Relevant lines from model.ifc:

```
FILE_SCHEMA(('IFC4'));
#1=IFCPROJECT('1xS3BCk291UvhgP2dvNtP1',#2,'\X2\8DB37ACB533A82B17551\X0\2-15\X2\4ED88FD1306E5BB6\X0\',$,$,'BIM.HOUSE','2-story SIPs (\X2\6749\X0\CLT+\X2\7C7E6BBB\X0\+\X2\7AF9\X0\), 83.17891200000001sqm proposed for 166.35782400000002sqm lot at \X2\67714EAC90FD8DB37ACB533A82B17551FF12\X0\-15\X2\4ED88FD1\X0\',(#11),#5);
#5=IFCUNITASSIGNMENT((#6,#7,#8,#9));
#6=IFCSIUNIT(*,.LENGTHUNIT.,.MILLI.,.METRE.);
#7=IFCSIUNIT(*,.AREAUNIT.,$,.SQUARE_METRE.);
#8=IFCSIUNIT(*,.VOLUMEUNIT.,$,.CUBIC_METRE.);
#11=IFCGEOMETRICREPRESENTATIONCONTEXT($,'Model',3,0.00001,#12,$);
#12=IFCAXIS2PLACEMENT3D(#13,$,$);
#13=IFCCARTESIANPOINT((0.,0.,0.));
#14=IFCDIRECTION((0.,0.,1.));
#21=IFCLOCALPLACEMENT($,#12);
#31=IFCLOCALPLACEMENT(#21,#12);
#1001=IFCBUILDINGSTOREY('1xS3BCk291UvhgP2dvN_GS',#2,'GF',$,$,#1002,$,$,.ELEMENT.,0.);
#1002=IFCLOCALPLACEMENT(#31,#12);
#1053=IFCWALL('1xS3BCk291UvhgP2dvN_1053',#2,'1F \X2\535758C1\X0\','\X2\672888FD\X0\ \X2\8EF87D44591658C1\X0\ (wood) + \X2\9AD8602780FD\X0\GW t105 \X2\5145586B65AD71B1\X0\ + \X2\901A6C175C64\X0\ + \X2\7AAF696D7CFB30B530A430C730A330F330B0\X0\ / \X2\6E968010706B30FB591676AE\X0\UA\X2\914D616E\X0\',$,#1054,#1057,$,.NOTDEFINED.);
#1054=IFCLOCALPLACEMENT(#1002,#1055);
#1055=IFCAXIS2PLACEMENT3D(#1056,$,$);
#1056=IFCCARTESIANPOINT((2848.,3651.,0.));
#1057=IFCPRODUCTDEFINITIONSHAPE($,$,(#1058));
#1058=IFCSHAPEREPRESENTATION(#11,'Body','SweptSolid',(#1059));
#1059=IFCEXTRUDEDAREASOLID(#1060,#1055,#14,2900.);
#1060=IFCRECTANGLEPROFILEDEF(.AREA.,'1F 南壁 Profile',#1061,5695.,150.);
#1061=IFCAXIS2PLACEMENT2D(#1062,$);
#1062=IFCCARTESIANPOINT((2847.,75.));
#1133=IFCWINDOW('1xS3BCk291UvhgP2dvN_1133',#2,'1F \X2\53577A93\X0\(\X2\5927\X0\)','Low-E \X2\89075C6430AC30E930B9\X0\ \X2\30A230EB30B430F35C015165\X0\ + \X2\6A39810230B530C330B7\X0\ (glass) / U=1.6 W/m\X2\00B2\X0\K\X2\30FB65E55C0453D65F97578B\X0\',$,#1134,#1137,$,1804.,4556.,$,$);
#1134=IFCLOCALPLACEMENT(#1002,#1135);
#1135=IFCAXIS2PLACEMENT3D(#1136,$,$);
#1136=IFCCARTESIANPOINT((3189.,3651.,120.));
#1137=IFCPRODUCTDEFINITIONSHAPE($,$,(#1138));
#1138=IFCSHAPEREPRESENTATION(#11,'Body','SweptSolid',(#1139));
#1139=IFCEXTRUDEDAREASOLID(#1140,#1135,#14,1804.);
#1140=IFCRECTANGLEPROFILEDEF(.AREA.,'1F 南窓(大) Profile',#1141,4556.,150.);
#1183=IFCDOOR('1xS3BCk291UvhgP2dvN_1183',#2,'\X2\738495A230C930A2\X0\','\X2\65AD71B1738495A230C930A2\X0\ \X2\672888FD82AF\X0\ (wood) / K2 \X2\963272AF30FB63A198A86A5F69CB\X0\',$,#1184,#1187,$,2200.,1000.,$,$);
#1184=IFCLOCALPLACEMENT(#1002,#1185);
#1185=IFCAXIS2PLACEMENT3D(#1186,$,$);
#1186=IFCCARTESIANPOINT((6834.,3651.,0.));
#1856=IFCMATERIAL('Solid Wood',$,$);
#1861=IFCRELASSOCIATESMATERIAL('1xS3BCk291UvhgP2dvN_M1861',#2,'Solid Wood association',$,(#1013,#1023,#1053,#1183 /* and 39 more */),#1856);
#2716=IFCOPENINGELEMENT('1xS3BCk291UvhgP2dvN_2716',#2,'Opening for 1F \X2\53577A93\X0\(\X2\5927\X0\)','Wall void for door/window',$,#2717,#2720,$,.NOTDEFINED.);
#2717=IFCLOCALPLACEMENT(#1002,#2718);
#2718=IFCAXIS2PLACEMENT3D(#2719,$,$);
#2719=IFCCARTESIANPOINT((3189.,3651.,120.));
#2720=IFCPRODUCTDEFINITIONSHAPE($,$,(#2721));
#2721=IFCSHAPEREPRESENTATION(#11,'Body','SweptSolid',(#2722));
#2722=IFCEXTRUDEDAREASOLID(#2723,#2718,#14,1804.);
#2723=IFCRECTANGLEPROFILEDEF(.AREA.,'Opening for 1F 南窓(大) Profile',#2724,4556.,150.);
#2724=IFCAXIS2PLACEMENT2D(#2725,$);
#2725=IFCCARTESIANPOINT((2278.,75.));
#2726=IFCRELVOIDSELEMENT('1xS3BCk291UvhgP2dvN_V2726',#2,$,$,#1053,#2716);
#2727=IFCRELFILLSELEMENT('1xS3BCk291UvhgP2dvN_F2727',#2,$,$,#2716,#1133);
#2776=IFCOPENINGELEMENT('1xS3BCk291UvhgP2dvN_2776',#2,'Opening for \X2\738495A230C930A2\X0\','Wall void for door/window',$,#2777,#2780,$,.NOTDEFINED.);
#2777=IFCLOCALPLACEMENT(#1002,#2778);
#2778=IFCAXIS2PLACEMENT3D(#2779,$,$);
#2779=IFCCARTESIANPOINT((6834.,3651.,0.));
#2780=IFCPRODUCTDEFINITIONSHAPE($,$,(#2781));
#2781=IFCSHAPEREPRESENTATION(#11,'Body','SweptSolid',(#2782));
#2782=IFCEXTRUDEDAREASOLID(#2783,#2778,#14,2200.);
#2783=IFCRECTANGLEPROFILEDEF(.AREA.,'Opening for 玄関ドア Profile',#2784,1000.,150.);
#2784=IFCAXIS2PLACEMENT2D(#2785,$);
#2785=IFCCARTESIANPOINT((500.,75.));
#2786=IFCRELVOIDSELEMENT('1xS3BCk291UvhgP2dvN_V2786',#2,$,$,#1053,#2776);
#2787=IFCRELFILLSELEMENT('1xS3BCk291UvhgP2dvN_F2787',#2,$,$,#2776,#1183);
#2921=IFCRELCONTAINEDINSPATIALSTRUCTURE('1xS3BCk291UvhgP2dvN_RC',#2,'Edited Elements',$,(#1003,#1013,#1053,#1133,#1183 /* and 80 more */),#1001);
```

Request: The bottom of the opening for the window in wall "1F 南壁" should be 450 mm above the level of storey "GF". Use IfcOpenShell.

```python
import numpy as np
import ifcopenshell
import ifcopenshell.api.geometry
import ifcopenshell.geom
import ifcopenshell.util.element
import ifcopenshell.util.placement
import ifcopenshell.util.shape
import ifcopenshell.util.unit

model = ifcopenshell.open("model.ifc")
unit_scale = ifcopenshell.util.unit.calculate_unit_scale(model)

window = model.by_id(1133)
opening = window.FillsVoids[0].RelatingOpeningElement
storey = ifcopenshell.util.element.get_container(window, ifc_class="IfcBuildingStorey")
level = ifcopenshell.util.placement.get_local_placement(storey.ObjectPlacement)[2, 3]

# The opening's origin need not be at the sill, so measure its lowest point.
shape = ifcopenshell.geom.create_shape(ifcopenshell.geom.settings(), opening)
bottom = ifcopenshell.util.shape.get_shape_bottom_elevation(shape, shape.geometry) / unit_scale
dz = level + 0.45 / unit_scale - bottom

shift = np.array([0.0, 0.0, dz])
# The window is not placed relative to its opening, so move both.
for product in (opening, window):
    matrix = ifcopenshell.util.placement.get_local_placement(product.ObjectPlacement)
    matrix[:3, 3] += shift
    ifcopenshell.api.geometry.edit_object_placement(model, product=product, matrix=matrix, is_si=False)

print(f"moved by {dz * unit_scale:+.3f} m")

model.write("model_rev.ifc")
```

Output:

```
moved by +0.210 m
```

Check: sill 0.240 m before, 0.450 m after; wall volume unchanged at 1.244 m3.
